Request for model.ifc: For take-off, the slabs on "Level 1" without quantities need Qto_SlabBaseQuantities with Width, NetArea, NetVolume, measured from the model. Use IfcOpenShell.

First a look at what the model holds.

```python
import ifcopenshell
import ifcopenshell.util.element
import ifcopenshell.util.unit

model = ifcopenshell.open("model.ifc")
print(model.schema)
for unit_type in ("LENGTHUNIT", "AREAUNIT", "VOLUMEUNIT"):
    print(unit_type, ifcopenshell.util.unit.calculate_unit_scale(model, unit_type))
storey = next(s for s in model.by_type("IfcBuildingStorey") if s.Name == "Level 1")
slabs = [e for e in ifcopenshell.util.element.get_decomposition(storey) if e.is_a("IfcSlab")]
for e in sorted(slabs, key=lambda e: e.id()):
    print(e.id(), e.is_a(), e.Name, list(ifcopenshell.util.element.get_psets(e, qtos_only=True)), sep=" | ")
```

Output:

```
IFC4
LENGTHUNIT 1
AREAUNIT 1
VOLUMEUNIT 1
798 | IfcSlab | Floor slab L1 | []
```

```python
import ifcopenshell
import ifcopenshell.api.pset
import ifcopenshell.geom
import ifcopenshell.util.element
import ifcopenshell.util.shape
import ifcopenshell.util.unit

model = ifcopenshell.open("model.ifc")
unit_scale = ifcopenshell.util.unit.calculate_unit_scale(model)
area_scale = ifcopenshell.util.unit.calculate_unit_scale(model, "AREAUNIT")
volume_scale = ifcopenshell.util.unit.calculate_unit_scale(model, "VOLUMEUNIT")
settings = ifcopenshell.geom.settings()

storey = next(s for s in model.by_type("IfcBuildingStorey") if s.Name == "Level 1")
slabs = [e for e in ifcopenshell.util.element.get_decomposition(storey) if e.is_a("IfcSlab")]

for e in sorted(slabs, key=lambda e: e.id()):
    if ifcopenshell.util.element.get_psets(e, qtos_only=True, should_inherit=False):
        continue
    # Geometry comes back in metres, in the element's own axes.
    shape = ifcopenshell.geom.create_shape(settings, e)
    values = {
        "Width": ifcopenshell.util.shape.get_z(shape.geometry) / unit_scale,
        "NetArea": ifcopenshell.util.shape.get_footprint_area(shape.geometry) / area_scale,
        "NetVolume": ifcopenshell.util.shape.get_volume(shape.geometry) / volume_scale,
    }
    qto = ifcopenshell.api.pset.add_qto(model, product=e, name="Qto_SlabBaseQuantities")
    ifcopenshell.api.pset.edit_qto(model, qto=qto, properties=values)
    print(e.id(), {k: round(v, 3) for k, v in values.items()})

model.write("model-out.ifc")
```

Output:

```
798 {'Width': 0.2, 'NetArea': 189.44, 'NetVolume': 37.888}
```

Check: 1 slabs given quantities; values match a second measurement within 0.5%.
